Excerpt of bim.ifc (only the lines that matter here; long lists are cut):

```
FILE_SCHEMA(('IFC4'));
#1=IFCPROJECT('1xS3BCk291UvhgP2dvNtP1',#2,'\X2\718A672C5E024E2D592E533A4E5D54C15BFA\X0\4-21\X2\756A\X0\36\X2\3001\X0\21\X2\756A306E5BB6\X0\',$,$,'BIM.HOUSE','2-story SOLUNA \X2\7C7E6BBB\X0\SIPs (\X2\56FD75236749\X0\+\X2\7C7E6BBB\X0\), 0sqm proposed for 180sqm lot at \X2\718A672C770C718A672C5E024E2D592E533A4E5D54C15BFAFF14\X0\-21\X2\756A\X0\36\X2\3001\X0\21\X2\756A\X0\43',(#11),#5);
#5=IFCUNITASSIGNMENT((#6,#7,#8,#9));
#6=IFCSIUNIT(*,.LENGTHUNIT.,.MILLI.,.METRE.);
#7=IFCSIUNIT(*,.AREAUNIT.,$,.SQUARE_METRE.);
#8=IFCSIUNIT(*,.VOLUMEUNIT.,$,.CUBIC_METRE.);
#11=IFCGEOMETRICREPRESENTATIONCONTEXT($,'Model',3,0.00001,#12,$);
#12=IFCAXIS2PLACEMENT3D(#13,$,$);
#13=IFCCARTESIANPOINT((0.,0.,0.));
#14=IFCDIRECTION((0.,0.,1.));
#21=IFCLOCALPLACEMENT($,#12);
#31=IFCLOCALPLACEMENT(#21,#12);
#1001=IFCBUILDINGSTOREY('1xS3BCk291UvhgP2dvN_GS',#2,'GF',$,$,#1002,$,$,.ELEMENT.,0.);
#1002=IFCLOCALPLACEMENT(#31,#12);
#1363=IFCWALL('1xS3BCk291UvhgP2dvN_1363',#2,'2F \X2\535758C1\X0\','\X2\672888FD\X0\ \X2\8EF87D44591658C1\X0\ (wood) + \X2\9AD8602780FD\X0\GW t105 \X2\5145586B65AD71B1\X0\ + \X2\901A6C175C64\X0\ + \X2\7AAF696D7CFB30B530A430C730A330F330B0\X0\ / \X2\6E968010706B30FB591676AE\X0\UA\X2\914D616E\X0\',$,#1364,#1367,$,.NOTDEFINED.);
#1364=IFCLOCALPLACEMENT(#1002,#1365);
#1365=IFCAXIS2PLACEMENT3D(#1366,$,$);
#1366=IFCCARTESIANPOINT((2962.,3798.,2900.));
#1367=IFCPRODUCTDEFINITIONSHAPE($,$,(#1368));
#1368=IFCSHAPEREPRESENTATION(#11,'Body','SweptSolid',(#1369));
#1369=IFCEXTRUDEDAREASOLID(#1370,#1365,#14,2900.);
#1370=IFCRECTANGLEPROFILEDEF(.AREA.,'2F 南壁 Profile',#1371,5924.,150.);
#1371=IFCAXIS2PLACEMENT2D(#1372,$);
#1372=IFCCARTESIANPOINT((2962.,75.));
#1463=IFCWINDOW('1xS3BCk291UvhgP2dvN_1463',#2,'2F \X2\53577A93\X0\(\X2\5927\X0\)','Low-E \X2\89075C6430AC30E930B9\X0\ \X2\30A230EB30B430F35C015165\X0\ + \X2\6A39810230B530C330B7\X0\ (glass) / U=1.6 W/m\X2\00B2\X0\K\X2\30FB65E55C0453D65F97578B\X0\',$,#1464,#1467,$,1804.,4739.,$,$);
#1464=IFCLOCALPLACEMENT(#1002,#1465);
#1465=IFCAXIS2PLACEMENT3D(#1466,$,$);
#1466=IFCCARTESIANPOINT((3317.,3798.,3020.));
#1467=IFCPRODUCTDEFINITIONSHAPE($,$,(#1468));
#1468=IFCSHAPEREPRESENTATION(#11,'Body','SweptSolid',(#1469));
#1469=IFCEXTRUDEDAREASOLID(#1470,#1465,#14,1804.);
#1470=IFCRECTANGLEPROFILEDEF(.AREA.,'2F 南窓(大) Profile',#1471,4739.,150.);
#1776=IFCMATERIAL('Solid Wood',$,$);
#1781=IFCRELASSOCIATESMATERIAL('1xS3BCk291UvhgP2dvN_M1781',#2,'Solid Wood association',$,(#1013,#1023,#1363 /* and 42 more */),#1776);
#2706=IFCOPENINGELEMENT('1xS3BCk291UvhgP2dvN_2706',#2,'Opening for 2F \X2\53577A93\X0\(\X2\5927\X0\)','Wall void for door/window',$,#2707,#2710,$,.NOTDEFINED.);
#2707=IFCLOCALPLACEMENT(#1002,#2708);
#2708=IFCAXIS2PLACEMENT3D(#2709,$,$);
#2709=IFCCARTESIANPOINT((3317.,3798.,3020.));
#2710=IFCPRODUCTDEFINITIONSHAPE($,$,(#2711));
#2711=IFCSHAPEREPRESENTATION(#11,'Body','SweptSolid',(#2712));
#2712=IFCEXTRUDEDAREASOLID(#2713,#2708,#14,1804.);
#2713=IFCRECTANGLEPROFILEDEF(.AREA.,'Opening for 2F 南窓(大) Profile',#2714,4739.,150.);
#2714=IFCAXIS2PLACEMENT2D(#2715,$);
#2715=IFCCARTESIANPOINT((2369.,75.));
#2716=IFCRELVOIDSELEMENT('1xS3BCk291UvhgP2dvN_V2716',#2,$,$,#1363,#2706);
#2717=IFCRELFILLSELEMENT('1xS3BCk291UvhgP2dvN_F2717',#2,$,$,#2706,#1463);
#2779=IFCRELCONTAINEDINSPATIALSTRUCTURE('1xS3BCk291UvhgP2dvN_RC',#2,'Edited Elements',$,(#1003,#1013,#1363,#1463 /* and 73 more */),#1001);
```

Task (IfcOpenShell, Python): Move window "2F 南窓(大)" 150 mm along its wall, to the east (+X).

```python
import ifcopenshell
import ifcopenshell.api.geometry
import ifcopenshell.util.placement

model = ifcopenshell.open("bim.ifc")

window = model.by_id(1463)
opening = window.FillsVoids[0].RelatingOpeningElement
wall = opening.VoidsElements[0].RelatingBuildingElement

wall_matrix = ifcopenshell.util.placement.get_local_placement(wall.ObjectPlacement)
shift = wall_matrix[:3, 0] * 150.0
before = ifcopenshell.util.placement.get_local_placement(window.ObjectPlacement)[:3, 3].copy()

# The window is not placed relative to its opening, so move both.
for product in (opening, window):
    matrix = ifcopenshell.util.placement.get_local_placement(product.ObjectPlacement)
    matrix[:3, 3] += shift
    ifcopenshell.api.geometry.edit_object_placement(model, product=product, matrix=matrix, is_si=False)

after = ifcopenshell.util.placement.get_local_placement(window.ObjectPlacement)[:3, 3]
print("window moved by", (after - before).round(3) + 0.0)

model.write("bim_edited.ifc")
```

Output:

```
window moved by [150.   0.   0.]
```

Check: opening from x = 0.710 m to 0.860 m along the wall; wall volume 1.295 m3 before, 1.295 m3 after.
